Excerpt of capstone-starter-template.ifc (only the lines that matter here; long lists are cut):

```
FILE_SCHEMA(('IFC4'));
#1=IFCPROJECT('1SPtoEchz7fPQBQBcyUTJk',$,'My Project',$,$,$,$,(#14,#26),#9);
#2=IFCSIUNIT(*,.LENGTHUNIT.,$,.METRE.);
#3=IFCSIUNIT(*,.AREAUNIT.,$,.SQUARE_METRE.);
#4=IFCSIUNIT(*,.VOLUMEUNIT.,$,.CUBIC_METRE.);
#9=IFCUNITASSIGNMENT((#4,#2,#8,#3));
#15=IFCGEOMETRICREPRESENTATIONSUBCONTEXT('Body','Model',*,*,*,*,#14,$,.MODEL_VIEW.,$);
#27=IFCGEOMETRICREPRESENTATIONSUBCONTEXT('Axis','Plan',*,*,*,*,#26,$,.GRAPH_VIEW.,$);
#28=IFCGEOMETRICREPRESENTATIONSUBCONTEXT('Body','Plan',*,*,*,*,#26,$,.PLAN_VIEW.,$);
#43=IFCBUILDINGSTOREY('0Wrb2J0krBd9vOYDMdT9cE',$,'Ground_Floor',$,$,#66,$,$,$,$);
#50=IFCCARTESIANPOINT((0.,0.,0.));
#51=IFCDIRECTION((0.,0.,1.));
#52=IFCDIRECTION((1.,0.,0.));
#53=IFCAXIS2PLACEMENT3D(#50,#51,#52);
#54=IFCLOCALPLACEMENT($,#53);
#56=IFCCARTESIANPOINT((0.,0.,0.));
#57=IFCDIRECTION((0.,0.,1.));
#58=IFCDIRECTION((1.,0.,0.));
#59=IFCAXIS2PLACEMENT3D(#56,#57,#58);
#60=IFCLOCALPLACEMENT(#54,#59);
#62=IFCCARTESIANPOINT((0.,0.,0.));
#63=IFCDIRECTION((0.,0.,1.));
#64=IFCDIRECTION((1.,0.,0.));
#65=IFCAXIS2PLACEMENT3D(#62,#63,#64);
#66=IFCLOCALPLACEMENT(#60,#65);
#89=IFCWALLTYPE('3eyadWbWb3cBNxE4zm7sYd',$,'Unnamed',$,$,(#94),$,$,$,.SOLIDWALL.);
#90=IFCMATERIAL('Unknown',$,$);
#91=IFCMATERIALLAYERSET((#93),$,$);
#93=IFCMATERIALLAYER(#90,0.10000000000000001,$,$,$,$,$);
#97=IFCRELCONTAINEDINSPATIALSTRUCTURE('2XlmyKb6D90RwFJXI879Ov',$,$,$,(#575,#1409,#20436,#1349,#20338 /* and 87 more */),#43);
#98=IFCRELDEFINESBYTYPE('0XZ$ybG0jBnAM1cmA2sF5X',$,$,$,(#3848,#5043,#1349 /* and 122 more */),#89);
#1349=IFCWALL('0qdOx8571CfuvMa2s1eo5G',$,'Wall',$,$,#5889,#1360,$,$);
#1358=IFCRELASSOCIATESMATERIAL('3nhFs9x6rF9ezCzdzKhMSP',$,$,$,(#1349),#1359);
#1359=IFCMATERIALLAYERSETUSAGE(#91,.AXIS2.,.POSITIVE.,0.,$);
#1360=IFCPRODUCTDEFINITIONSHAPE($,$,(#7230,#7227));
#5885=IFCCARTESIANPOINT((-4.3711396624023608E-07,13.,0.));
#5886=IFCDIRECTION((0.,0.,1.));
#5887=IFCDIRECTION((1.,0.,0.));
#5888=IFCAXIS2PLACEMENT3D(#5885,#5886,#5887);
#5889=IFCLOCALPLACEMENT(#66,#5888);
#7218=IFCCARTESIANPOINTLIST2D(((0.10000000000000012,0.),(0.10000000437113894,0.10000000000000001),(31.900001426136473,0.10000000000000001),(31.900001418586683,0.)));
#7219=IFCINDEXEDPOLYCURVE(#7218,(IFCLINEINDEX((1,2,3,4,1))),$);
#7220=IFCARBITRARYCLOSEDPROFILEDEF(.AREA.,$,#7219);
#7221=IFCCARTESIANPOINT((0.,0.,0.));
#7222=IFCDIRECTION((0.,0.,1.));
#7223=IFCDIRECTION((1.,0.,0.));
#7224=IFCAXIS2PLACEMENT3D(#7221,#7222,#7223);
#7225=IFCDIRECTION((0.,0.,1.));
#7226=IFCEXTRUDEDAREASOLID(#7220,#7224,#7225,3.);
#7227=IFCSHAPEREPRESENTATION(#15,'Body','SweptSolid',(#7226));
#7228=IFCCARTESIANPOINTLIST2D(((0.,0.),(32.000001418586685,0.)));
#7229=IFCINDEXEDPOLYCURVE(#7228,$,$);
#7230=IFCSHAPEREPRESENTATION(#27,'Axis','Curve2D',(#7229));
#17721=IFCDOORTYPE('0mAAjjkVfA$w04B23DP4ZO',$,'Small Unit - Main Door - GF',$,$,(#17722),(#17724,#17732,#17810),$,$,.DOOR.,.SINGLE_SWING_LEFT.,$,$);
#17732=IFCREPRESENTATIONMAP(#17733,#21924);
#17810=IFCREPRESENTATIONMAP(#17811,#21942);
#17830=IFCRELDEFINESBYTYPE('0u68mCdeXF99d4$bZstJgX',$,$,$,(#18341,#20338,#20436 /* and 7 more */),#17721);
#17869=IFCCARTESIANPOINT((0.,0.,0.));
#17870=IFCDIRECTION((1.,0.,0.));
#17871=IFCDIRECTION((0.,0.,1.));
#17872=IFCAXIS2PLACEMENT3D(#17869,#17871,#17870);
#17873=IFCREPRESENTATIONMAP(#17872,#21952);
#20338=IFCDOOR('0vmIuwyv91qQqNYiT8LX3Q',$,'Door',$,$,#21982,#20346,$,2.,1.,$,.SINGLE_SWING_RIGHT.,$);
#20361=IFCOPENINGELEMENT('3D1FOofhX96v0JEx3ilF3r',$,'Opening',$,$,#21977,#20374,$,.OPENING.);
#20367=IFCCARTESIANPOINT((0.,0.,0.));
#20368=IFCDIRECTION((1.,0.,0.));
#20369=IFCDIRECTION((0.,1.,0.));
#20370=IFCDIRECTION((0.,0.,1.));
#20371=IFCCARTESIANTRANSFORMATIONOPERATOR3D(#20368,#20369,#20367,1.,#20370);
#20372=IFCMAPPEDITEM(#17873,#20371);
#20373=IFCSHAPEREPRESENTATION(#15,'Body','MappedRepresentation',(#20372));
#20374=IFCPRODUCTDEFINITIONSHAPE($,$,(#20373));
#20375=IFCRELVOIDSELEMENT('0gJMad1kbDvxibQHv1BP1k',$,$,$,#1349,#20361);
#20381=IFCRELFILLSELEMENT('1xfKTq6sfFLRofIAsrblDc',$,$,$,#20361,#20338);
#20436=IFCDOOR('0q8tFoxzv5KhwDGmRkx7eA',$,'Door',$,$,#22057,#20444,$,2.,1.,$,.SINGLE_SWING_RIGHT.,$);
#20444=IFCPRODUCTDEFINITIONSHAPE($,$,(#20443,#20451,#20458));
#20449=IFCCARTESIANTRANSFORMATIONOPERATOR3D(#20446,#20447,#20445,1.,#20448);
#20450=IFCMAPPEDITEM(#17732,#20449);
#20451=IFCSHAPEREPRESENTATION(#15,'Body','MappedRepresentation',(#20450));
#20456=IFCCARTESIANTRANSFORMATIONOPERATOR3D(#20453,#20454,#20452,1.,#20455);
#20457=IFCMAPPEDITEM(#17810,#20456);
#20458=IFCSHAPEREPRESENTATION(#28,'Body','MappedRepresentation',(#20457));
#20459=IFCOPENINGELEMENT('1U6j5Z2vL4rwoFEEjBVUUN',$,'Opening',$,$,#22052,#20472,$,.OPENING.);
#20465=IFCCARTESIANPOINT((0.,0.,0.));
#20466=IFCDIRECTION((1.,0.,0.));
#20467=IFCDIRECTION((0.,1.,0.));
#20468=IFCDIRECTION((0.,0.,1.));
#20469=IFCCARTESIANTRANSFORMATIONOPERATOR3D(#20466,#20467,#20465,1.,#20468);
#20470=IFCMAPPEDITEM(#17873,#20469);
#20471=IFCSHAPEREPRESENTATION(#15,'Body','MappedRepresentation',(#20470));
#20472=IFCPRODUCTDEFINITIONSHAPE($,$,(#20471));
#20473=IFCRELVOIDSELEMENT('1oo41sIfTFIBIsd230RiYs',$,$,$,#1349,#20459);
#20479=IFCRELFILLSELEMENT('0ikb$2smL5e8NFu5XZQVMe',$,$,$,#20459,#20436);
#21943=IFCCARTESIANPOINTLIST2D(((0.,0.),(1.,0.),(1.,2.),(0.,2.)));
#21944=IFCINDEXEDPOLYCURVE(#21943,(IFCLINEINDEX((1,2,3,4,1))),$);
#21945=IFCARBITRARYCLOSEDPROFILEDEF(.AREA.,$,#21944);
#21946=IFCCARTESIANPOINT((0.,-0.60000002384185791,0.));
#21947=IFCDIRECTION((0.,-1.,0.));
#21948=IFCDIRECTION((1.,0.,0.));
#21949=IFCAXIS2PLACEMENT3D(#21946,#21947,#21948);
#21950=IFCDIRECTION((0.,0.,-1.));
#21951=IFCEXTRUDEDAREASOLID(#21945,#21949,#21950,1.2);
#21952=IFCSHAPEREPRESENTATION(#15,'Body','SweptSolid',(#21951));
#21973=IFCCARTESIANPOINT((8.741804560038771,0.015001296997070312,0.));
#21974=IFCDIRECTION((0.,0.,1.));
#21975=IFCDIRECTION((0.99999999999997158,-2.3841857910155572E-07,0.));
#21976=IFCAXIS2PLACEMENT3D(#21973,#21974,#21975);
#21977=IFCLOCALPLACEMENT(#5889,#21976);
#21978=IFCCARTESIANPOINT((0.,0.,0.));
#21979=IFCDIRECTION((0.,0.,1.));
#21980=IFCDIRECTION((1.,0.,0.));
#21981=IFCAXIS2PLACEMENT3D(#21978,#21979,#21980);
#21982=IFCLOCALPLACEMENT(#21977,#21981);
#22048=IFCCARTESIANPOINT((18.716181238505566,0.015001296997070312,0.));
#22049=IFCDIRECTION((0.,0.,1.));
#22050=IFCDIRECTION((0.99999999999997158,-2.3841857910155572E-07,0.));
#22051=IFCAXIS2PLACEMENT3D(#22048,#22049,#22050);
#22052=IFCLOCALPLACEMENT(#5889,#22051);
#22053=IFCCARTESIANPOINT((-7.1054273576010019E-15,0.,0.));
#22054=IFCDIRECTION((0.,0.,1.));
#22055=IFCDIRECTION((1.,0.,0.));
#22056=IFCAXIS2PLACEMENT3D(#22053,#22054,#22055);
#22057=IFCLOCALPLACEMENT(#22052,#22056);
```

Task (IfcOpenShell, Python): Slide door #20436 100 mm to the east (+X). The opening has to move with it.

```python
import ifcopenshell
import ifcopenshell.api.geometry
import ifcopenshell.util.placement
import ifcopenshell.util.unit

model = ifcopenshell.open("capstone-starter-template.ifc")
unit_scale = ifcopenshell.util.unit.calculate_unit_scale(model)

door = model.by_guid("0q8tFoxzv5KhwDGmRkx7eA")
opening = door.FillsVoids[0].RelatingOpeningElement
wall = opening.VoidsElements[0].RelatingBuildingElement

wall_matrix = ifcopenshell.util.placement.get_local_placement(wall.ObjectPlacement)
shift = wall_matrix[:3, 0] * 0.1 / unit_scale
before = ifcopenshell.util.placement.get_local_placement(door.ObjectPlacement)[:3, 3].copy()

# The door is placed relative to its opening, so it follows when the opening moves.
matrix = ifcopenshell.util.placement.get_local_placement(opening.ObjectPlacement)
matrix[:3, 3] += shift
ifcopenshell.api.geometry.edit_object_placement(
    model, product=opening, matrix=matrix, is_si=False, should_transform_children=True
)

after = ifcopenshell.util.placement.get_local_placement(door.ObjectPlacement)[:3, 3]
print("door moved by", (after - before).round(3) + 0.0)

model.write("capstone-starter-template_updated.ifc")
```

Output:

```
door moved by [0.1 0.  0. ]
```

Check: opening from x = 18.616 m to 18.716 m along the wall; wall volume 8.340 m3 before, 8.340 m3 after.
